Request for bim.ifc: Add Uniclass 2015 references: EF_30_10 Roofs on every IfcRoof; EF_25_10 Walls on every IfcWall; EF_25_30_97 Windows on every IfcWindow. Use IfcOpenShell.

First a look at what the model holds.

```python
import ifcopenshell

model = ifcopenshell.open("bim.ifc")
print(model.schema)
print("classifications:", [c.Name for c in model.by_type("IfcClassification")])
for ifc_class in ("IfcDoor", "IfcRoof", "IfcStair", "IfcWall", "IfcWindow"):
    print(ifc_class, len(model.by_type(ifc_class)))
```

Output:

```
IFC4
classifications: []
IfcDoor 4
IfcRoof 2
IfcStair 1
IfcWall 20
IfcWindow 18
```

```python
import ifcopenshell
import ifcopenshell.api.classification

model = ifcopenshell.open("bim.ifc")

system = ifcopenshell.api.classification.add_classification(model, classification="Uniclass 2015")

codes = {
    "IfcRoof": ("EF_30_10", "Roofs"),
    "IfcWall": ("EF_25_10", "Walls"),
    "IfcWindow": ("EF_25_30_97", "Windows"),
}
for ifc_class, (code, name) in codes.items():
    products = model.by_type(ifc_class)
    ifcopenshell.api.classification.add_reference(
        model, products=products, classification=system, identification=code, name=name
    )
    print(code, len(products))

model.write("bim_rev.ifc")
```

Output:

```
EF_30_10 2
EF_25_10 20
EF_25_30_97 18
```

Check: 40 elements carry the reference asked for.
